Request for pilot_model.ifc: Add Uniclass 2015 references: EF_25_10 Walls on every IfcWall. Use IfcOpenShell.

First a look at what the model holds.

```python
import ifcopenshell

model = ifcopenshell.open("pilot_model.ifc")
print(model.schema)
print("classifications:", [c.Name for c in model.by_type("IfcClassification")])
for ifc_class in ("IfcDoor", "IfcRoof", "IfcStair", "IfcWall", "IfcWindow"):
    print(ifc_class, len(model.by_type(ifc_class)))
```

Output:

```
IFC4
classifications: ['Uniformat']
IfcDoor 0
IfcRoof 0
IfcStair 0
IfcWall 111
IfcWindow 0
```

```python
import ifcopenshell
import ifcopenshell.api.classification

model = ifcopenshell.open("pilot_model.ifc")

system = ifcopenshell.api.classification.add_classification(model, classification="Uniclass 2015")

codes = {
    "IfcWall": ("EF_25_10", "Walls"),
}
for ifc_class, (code, name) in codes.items():
    products = model.by_type(ifc_class)
    ifcopenshell.api.classification.add_reference(
        model, products=products, classification=system, identification=code, name=name
    )
    print(code, len(products))

model.write("pilot_model_rev.ifc")
```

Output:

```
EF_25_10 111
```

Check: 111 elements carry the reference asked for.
